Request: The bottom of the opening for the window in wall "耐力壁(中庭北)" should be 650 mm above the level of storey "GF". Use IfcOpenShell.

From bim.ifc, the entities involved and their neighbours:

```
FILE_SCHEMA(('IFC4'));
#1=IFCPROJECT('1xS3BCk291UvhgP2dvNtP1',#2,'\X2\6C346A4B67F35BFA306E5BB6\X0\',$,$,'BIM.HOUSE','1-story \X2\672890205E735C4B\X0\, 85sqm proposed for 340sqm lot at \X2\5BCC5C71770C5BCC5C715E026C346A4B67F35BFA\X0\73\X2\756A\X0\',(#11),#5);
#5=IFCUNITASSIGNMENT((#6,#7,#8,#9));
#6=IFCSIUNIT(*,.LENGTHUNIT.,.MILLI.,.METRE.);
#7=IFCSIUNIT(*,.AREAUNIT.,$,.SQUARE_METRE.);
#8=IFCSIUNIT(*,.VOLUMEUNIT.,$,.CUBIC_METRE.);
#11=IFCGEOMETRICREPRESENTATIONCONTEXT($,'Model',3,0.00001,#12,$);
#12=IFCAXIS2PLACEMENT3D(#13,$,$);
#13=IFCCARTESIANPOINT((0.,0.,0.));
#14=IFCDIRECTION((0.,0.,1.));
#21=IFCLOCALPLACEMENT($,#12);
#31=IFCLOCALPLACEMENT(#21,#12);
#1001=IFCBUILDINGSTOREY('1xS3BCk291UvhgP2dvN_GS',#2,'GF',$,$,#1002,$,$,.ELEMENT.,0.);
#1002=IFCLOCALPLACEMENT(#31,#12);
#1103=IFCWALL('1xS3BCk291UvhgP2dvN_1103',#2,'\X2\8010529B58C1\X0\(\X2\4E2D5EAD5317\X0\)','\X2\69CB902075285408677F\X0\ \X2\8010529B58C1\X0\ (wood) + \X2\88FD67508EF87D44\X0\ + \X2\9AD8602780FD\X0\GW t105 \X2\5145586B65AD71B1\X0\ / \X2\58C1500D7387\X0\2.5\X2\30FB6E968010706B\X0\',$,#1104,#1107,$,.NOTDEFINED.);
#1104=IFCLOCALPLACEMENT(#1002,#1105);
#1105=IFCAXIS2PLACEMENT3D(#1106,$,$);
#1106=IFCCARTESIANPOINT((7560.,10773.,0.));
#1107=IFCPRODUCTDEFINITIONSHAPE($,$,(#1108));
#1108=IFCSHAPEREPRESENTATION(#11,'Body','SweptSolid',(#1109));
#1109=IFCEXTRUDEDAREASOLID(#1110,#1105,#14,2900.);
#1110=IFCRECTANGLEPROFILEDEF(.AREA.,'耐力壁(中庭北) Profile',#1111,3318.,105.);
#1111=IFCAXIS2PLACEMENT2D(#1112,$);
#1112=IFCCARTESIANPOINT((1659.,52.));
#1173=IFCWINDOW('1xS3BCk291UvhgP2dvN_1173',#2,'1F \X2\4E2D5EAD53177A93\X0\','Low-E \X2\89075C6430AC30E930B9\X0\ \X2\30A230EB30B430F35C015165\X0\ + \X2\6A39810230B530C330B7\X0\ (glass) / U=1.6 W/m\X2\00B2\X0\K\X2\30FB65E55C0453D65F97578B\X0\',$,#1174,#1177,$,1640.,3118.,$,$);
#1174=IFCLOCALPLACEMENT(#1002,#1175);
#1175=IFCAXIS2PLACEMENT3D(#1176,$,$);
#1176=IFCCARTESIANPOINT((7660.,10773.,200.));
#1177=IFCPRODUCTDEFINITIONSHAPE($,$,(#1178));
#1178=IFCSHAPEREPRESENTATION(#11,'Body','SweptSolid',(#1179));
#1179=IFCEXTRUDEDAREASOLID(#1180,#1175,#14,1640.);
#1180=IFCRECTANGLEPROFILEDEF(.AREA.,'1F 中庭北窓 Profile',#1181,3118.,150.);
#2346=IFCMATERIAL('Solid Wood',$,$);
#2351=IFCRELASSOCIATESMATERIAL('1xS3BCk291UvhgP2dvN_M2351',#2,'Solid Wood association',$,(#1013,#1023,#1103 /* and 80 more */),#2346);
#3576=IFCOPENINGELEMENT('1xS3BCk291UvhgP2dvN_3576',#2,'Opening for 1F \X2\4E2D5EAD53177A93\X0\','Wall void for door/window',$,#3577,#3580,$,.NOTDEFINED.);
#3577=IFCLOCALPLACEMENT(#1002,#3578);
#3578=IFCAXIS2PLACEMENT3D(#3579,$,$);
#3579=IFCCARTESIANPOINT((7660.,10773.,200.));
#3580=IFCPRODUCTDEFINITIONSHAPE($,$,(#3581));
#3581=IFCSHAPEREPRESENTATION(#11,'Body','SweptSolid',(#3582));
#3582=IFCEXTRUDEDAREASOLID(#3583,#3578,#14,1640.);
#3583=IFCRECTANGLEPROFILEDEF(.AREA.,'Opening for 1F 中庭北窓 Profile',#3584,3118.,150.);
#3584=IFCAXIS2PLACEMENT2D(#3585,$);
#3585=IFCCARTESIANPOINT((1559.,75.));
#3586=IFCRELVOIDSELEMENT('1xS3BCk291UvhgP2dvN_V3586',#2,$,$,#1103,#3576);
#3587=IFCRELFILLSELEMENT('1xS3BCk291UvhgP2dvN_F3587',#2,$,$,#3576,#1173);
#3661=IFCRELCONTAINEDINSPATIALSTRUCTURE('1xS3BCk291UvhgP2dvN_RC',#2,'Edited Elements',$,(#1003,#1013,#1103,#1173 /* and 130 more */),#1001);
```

```python
import numpy as np
import ifcopenshell
import ifcopenshell.api.geometry
import ifcopenshell.geom
import ifcopenshell.util.element
import ifcopenshell.util.placement
import ifcopenshell.util.shape
import ifcopenshell.util.unit

model = ifcopenshell.open("bim.ifc")
unit_scale = ifcopenshell.util.unit.calculate_unit_scale(model)

window = model.by_guid("1xS3BCk291UvhgP2dvN_1173")
opening = window.FillsVoids[0].RelatingOpeningElement
storey = ifcopenshell.util.element.get_container(window, ifc_class="IfcBuildingStorey")
level = ifcopenshell.util.placement.get_local_placement(storey.ObjectPlacement)[2, 3]

# The opening's origin need not be at the sill, so measure its lowest point.
shape = ifcopenshell.geom.create_shape(ifcopenshell.geom.settings(), opening)
bottom = ifcopenshell.util.shape.get_shape_bottom_elevation(shape, shape.geometry) / unit_scale
dz = level + 0.65 / unit_scale - bottom

shift = np.array([0.0, 0.0, dz])
# The window is not placed relative to its opening, so move both.
for product in (opening, window):
    matrix = ifcopenshell.util.placement.get_local_placement(product.ObjectPlacement)
    matrix[:3, 3] += shift
    ifcopenshell.api.geometry.edit_object_placement(model, product=product, matrix=matrix, is_si=False)

print(f"moved by {dz * unit_scale:+.3f} m")

model.write("bim_rev.ifc")
```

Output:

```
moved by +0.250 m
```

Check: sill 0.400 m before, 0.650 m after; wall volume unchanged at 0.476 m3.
